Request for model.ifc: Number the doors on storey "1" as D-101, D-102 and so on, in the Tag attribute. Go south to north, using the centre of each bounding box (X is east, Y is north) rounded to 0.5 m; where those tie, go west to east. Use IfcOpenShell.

First a look at what the model holds.

```python
import ifcopenshell
import ifcopenshell.util.element
import ifcopenshell.util.placement

model = ifcopenshell.open("model.ifc")
print(model.schema)
storey = next(s for s in model.by_type("IfcBuildingStorey") if s.Name == "1")
doors = [e for e in ifcopenshell.util.element.get_decomposition(storey) if e.is_a("IfcDoor")]
for e in sorted(doors, key=lambda e: e.id()):
    origin = ifcopenshell.util.placement.get_local_placement(e.ObjectPlacement)[:3, 3]
    print(e.id(), e.Tag, e.Name, origin.round(2) + 0.0, sep=" | ")
```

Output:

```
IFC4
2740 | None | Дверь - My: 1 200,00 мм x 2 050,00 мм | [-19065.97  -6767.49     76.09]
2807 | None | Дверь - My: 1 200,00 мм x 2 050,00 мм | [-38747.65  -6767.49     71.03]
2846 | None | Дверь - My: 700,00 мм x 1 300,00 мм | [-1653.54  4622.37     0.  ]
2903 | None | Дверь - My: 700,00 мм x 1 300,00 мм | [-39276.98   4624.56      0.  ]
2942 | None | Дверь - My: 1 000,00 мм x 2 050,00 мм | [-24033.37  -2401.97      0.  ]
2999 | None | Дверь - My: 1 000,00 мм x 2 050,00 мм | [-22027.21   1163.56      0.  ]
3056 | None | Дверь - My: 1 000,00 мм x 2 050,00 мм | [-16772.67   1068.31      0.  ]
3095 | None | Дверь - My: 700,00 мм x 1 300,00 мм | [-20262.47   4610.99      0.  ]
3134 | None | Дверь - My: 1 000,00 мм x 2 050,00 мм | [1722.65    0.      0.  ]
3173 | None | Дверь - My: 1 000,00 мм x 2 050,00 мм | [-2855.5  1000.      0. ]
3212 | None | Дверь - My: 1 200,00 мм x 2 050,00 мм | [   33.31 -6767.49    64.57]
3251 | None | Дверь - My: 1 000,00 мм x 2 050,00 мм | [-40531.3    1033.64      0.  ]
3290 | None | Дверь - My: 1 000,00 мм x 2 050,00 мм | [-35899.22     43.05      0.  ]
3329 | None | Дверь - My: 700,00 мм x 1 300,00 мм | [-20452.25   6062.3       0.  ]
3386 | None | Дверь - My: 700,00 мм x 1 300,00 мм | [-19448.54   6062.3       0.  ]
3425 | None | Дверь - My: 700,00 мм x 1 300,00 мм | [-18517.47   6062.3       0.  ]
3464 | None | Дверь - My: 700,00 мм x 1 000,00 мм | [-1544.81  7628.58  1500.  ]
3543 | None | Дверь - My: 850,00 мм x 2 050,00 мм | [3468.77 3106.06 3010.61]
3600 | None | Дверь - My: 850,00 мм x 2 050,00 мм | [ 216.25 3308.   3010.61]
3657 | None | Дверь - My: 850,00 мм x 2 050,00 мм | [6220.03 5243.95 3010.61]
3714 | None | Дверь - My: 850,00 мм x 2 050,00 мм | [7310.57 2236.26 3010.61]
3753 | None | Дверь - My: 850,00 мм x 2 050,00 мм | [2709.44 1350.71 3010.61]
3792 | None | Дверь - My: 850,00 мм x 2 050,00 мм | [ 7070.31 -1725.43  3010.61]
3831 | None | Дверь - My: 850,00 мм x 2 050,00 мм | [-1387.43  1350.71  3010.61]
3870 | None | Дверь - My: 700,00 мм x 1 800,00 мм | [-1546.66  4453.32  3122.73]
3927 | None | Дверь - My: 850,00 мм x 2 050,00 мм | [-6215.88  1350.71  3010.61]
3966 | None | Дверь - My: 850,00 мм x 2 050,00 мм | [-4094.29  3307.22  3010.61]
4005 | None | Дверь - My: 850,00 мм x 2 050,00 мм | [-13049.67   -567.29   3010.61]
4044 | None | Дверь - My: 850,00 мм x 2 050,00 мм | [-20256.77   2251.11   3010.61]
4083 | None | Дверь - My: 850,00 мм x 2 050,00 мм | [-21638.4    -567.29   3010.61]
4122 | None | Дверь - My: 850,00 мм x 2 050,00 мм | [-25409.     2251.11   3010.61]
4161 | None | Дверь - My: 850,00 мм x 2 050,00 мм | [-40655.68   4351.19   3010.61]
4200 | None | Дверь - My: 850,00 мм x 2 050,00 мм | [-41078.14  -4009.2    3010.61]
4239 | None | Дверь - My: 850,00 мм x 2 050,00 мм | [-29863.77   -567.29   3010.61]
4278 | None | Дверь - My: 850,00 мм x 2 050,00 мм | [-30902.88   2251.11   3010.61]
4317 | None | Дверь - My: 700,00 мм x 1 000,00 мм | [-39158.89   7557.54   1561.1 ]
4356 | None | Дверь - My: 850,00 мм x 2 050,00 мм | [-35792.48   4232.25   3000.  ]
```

```python
import ifcopenshell
import ifcopenshell.geom
import ifcopenshell.util.element
import ifcopenshell.util.shape

model = ifcopenshell.open("model.ifc")
settings = ifcopenshell.geom.settings()
settings.set("use-world-coords", True)


def centre(element):
    shape = ifcopenshell.geom.create_shape(settings, element)
    return ifcopenshell.util.shape.get_bbox_centroid(shape.geometry)


storey = next(s for s in model.by_type("IfcBuildingStorey") if s.Name == "1")
doors = [e for e in ifcopenshell.util.element.get_decomposition(storey) if e.is_a("IfcDoor")]

# Insertion points can sit at a corner or the storey origin, so sort by the geometry (in metres).
centres = {e: centre(e) for e in doors}
doors.sort(key=lambda e: (round(centres[e][1] / 0.5), centres[e][0]))

for i, e in enumerate(doors, start=1):
    number = f"D-1{i:02d}"
    e.Tag = number
    print(e.id(), number)

model.write("model-out.ifc")
```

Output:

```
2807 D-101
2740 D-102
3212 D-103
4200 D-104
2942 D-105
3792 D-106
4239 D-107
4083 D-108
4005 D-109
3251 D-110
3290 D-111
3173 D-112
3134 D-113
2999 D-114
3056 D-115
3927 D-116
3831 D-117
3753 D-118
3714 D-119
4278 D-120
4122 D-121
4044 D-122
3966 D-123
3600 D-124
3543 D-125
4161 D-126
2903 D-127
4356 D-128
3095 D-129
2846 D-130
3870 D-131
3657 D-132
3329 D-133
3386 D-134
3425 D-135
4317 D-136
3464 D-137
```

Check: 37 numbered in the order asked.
